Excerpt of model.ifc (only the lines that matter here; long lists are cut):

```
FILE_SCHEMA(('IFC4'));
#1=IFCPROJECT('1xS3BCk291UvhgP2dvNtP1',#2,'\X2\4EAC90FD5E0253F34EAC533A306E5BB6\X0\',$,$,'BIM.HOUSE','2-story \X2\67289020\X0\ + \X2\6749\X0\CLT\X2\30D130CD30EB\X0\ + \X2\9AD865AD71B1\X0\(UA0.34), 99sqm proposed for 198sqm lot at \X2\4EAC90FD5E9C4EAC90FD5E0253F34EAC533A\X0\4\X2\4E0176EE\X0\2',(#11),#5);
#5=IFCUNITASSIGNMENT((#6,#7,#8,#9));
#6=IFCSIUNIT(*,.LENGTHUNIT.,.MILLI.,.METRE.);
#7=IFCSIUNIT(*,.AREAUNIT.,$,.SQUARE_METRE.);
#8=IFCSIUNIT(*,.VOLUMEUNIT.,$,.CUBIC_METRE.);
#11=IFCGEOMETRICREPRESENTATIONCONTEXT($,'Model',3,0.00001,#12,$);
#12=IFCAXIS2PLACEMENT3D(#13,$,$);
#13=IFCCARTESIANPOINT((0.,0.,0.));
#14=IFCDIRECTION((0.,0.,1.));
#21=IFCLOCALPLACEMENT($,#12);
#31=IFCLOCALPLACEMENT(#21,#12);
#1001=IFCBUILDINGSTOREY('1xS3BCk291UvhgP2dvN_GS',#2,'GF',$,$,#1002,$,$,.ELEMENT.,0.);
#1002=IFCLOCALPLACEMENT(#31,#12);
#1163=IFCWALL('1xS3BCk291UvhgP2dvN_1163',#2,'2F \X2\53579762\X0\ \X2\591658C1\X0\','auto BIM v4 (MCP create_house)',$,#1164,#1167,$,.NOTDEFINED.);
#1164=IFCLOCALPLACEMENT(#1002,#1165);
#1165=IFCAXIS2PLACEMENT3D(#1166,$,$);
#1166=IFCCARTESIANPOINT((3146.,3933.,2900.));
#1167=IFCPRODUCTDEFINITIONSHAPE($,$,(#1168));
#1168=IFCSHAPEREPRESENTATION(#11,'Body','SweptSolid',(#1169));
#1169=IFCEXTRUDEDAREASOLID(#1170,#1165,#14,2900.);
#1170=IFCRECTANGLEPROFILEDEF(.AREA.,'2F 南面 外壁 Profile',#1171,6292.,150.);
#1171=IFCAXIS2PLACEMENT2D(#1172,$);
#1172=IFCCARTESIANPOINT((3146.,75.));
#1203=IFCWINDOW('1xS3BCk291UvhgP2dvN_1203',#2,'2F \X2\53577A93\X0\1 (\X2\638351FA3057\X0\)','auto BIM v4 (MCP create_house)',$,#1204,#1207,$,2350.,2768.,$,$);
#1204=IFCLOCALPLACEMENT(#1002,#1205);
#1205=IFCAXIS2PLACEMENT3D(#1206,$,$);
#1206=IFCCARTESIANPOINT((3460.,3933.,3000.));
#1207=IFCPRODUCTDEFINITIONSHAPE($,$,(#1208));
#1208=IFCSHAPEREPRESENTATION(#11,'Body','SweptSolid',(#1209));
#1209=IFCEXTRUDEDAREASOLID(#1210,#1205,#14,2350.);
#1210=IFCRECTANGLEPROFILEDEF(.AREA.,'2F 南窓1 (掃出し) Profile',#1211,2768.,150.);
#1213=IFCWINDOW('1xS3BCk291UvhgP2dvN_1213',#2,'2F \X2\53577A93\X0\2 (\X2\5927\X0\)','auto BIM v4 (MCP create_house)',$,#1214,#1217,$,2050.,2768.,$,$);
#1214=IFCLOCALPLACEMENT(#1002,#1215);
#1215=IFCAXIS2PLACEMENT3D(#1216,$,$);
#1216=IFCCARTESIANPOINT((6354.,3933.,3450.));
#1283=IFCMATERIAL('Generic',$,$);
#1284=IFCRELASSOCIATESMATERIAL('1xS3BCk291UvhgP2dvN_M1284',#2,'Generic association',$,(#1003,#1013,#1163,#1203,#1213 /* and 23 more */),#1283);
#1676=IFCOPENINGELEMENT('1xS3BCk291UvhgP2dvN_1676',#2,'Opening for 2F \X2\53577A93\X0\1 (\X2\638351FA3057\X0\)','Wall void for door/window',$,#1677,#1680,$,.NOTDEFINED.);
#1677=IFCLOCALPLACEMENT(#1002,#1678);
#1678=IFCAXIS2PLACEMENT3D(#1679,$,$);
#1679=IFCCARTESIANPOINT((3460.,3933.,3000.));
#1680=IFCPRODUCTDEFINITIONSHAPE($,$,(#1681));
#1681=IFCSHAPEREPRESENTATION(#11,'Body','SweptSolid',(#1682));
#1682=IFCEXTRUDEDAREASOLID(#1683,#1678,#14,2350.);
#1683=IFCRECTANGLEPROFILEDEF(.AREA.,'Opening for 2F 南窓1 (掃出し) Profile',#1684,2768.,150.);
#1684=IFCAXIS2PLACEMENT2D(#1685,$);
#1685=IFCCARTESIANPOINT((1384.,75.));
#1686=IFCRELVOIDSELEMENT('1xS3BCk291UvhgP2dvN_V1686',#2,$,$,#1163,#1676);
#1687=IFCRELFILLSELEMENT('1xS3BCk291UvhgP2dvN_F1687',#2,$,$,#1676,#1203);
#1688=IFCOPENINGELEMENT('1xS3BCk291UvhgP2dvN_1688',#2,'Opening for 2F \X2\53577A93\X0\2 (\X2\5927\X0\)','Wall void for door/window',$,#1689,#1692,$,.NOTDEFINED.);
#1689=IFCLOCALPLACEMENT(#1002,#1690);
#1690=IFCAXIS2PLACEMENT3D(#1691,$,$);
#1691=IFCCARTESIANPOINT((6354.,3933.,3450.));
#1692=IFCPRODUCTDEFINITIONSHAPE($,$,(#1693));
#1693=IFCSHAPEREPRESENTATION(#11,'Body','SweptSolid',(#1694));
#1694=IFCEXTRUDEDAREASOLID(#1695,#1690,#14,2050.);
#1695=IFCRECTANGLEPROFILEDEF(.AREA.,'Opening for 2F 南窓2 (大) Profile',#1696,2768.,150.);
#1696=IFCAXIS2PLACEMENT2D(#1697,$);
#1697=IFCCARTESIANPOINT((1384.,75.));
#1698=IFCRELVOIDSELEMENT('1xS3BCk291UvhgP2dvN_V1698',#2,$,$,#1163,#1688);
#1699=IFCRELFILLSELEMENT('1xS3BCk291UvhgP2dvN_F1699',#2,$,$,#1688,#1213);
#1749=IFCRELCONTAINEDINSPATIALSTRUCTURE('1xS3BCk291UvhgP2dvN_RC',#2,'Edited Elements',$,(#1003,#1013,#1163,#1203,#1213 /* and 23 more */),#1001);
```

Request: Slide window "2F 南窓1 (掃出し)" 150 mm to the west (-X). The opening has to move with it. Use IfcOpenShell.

```python
import ifcopenshell
import ifcopenshell.api.geometry
import ifcopenshell.util.placement
import ifcopenshell.util.unit

model = ifcopenshell.open("model.ifc")
unit_scale = ifcopenshell.util.unit.calculate_unit_scale(model)

window = model.by_guid("1xS3BCk291UvhgP2dvN_1203")
opening = window.FillsVoids[0].RelatingOpeningElement
wall = opening.VoidsElements[0].RelatingBuildingElement

wall_matrix = ifcopenshell.util.placement.get_local_placement(wall.ObjectPlacement)
shift = wall_matrix[:3, 0] * -0.15 / unit_scale
before = ifcopenshell.util.placement.get_local_placement(window.ObjectPlacement)[:3, 3].copy()

# The window is not placed relative to its opening, so move both.
for product in (opening, window):
    matrix = ifcopenshell.util.placement.get_local_placement(product.ObjectPlacement)
    matrix[:3, 3] += shift
    ifcopenshell.api.geometry.edit_object_placement(model, product=product, matrix=matrix, is_si=False)

after = ifcopenshell.util.placement.get_local_placement(window.ObjectPlacement)[:3, 3]
print("window moved by", (after - before).round(3) + 0.0)

model.write("model_v2.ifc")
```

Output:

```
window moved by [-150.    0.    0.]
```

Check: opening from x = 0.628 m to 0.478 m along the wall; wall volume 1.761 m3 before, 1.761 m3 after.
